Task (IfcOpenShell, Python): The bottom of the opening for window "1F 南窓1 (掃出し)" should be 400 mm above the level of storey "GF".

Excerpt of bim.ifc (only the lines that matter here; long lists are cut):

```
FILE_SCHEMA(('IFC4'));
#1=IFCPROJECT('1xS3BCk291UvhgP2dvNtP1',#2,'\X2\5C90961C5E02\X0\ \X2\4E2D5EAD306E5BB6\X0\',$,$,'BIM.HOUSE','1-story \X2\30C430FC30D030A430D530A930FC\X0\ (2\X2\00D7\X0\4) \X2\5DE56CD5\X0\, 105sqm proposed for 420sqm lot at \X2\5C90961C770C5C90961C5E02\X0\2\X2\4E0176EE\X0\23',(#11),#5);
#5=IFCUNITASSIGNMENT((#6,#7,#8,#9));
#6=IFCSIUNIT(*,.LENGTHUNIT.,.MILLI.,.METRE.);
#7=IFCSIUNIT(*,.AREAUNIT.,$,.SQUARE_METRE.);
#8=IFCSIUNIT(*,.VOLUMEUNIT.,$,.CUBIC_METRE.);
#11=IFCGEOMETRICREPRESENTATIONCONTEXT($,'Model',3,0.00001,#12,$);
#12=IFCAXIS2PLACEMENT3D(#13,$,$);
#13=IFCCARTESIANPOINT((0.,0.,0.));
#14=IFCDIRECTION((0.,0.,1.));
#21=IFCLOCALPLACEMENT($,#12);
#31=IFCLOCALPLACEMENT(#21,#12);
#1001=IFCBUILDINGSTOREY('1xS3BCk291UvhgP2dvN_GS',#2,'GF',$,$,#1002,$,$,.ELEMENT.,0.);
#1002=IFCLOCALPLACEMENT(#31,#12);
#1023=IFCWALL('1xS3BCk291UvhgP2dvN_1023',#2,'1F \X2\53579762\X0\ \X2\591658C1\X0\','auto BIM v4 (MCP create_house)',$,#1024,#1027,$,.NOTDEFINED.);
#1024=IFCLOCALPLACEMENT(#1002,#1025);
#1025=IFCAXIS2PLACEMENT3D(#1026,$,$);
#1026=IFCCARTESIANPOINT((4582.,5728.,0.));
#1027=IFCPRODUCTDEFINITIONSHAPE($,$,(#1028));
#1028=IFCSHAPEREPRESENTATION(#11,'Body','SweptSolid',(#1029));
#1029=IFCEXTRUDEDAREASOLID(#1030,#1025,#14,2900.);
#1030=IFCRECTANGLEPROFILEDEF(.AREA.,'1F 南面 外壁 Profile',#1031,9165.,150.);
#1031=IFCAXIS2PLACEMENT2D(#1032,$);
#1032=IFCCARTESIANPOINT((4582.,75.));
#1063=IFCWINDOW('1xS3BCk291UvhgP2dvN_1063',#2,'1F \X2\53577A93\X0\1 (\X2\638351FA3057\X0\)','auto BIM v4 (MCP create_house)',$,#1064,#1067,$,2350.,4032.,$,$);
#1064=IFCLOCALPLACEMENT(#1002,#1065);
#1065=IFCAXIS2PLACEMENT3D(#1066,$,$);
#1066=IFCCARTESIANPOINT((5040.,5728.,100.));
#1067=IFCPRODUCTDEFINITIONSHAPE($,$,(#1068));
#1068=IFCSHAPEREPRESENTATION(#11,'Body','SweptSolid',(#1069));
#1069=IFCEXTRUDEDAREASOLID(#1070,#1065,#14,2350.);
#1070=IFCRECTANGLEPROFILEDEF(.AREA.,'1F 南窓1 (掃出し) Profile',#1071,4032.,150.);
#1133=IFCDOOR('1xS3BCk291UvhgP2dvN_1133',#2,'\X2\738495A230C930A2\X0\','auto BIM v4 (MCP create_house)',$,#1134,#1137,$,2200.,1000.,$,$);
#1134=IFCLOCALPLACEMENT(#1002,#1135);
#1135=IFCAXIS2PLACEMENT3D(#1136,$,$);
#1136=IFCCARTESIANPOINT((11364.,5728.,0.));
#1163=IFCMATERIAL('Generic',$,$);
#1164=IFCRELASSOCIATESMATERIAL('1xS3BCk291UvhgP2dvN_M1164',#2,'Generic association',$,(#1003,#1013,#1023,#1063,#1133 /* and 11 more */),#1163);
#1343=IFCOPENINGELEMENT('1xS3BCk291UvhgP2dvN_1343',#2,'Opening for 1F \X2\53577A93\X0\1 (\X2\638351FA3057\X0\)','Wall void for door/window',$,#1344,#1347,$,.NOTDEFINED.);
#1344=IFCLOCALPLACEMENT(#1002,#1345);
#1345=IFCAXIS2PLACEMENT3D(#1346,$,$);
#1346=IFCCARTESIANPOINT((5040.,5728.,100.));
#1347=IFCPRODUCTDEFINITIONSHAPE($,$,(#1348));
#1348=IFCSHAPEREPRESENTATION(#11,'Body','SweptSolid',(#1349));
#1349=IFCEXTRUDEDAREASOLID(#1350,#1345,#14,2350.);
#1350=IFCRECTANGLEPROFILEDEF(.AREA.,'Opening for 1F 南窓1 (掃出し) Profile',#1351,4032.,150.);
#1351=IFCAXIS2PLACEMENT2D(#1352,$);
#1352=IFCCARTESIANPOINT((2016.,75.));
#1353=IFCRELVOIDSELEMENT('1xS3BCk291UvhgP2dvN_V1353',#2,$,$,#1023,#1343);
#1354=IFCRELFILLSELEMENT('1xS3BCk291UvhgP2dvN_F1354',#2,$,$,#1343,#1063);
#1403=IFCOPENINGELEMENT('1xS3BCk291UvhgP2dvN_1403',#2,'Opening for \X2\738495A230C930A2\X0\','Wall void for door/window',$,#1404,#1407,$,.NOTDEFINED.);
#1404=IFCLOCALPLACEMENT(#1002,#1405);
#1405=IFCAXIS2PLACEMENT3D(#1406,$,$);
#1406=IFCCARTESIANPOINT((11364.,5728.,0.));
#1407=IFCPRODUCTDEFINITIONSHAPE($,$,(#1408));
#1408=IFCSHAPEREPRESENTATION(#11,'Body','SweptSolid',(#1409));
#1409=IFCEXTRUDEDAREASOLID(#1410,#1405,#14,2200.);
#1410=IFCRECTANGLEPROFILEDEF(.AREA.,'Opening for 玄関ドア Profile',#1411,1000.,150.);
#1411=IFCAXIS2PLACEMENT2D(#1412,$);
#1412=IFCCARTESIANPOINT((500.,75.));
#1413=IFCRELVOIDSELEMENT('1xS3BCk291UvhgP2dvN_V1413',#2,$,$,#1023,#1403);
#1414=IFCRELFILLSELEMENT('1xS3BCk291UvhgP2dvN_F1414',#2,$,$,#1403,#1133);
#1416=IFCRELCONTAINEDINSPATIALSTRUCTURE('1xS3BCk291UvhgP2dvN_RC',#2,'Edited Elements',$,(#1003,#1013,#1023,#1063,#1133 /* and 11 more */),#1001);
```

```python
import numpy as np
import ifcopenshell
import ifcopenshell.api.geometry
import ifcopenshell.geom
import ifcopenshell.util.element
import ifcopenshell.util.placement
import ifcopenshell.util.shape
import ifcopenshell.util.unit

model = ifcopenshell.open("bim.ifc")
unit_scale = ifcopenshell.util.unit.calculate_unit_scale(model)

window = model.by_guid("1xS3BCk291UvhgP2dvN_1063")
opening = window.FillsVoids[0].RelatingOpeningElement
storey = ifcopenshell.util.element.get_container(window, ifc_class="IfcBuildingStorey")
level = ifcopenshell.util.placement.get_local_placement(storey.ObjectPlacement)[2, 3]

# The opening's origin need not be at the sill, so measure its lowest point.
shape = ifcopenshell.geom.create_shape(ifcopenshell.geom.settings(), opening)
bottom = ifcopenshell.util.shape.get_shape_bottom_elevation(shape, shape.geometry) / unit_scale
dz = level + 400.0 - bottom

shift = np.array([0.0, 0.0, dz])
# The window is not placed relative to its opening, so move both.
for product in (opening, window):
    matrix = ifcopenshell.util.placement.get_local_placement(product.ObjectPlacement)
    matrix[:3, 3] += shift
    ifcopenshell.api.geometry.edit_object_placement(model, product=product, matrix=matrix, is_si=False)

print(f"moved by {dz * unit_scale:+.3f} m")

model.write("bim-out.ifc")
```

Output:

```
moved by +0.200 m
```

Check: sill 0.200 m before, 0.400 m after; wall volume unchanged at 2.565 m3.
